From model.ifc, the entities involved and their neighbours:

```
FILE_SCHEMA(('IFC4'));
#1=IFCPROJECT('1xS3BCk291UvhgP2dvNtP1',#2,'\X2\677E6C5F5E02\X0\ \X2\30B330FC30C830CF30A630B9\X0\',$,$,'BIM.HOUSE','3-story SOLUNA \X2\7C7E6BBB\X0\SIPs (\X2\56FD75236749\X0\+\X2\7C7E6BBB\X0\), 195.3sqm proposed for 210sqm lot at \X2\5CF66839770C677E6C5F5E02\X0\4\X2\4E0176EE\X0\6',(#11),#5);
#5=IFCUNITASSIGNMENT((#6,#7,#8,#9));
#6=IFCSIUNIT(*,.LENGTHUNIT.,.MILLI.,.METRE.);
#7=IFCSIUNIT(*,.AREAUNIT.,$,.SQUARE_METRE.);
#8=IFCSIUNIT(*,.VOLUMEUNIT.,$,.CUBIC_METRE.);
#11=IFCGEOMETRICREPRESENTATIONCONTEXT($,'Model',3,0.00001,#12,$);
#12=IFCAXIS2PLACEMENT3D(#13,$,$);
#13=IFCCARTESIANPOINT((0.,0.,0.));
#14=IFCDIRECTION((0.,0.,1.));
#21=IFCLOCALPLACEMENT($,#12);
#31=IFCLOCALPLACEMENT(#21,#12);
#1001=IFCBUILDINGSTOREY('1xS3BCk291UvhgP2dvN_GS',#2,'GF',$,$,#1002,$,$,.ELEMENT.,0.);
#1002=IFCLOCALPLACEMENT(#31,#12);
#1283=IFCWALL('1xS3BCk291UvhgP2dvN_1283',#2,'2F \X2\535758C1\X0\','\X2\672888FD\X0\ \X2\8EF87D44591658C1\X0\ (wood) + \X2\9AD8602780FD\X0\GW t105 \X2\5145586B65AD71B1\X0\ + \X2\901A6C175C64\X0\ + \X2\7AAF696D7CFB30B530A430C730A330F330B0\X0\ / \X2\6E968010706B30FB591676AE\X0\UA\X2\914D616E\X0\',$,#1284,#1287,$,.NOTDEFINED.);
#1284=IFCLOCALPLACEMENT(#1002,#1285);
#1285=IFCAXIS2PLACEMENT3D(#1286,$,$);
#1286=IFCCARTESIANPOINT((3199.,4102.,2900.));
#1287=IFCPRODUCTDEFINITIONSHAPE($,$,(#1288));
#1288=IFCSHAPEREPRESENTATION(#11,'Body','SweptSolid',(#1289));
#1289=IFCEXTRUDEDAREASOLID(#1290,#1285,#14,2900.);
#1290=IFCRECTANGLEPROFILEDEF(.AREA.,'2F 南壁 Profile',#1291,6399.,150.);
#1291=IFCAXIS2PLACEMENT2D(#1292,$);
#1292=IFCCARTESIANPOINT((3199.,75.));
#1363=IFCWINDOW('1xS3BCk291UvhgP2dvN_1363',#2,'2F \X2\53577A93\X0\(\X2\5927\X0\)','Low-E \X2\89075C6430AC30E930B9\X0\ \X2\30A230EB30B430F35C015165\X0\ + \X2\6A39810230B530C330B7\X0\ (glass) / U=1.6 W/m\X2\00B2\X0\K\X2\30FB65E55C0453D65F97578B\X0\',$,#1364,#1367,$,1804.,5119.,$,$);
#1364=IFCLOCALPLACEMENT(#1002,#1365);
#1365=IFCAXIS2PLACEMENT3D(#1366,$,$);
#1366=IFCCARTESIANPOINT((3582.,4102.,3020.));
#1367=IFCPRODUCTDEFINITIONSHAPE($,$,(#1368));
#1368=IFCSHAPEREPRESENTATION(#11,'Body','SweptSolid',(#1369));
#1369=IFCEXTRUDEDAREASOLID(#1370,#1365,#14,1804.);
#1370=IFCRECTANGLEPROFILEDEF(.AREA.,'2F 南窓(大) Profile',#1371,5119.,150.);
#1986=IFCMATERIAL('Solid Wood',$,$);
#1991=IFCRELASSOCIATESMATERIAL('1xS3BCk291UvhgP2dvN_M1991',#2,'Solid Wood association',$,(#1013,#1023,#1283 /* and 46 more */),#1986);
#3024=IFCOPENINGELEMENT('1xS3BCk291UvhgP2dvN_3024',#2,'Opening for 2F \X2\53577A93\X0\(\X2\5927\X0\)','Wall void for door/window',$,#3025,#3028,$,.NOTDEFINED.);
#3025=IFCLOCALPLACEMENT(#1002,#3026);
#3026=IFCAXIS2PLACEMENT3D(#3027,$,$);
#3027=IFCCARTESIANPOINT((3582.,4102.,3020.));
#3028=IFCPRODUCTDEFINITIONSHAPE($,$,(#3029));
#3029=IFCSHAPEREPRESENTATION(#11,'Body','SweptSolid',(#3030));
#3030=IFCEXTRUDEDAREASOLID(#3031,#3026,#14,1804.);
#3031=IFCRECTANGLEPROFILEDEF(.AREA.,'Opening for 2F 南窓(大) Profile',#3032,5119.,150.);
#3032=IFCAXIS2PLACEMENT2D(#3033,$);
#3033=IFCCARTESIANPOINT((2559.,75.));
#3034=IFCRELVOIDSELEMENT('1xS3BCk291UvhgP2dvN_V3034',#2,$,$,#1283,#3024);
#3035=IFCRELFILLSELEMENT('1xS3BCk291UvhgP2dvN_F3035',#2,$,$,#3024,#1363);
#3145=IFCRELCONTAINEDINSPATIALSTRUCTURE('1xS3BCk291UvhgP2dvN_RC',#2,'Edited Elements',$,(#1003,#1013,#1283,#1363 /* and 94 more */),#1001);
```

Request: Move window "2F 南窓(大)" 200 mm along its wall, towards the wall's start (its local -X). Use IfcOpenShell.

```python
import ifcopenshell
import ifcopenshell.api.geometry
import ifcopenshell.util.placement

model = ifcopenshell.open("model.ifc")

window = model.by_id(1363)
opening = window.FillsVoids[0].RelatingOpeningElement
wall = opening.VoidsElements[0].RelatingBuildingElement

wall_matrix = ifcopenshell.util.placement.get_local_placement(wall.ObjectPlacement)
shift = wall_matrix[:3, 0] * -200.0
before = ifcopenshell.util.placement.get_local_placement(window.ObjectPlacement)[:3, 3].copy()

# The window is not placed relative to its opening, so move both.
for product in (opening, window):
    matrix = ifcopenshell.util.placement.get_local_placement(product.ObjectPlacement)
    matrix[:3, 3] += shift
    ifcopenshell.api.geometry.edit_object_placement(model, product=product, matrix=matrix, is_si=False)

after = ifcopenshell.util.placement.get_local_placement(window.ObjectPlacement)[:3, 3]
print("window moved by", (after - before).round(3) + 0.0)

model.write("model_updated.ifc")
```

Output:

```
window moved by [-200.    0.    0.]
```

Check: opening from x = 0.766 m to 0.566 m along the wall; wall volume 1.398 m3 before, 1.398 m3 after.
